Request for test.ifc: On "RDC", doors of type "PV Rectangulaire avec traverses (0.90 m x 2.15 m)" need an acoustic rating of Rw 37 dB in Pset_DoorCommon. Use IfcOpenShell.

First a look at what the model holds.

```python
import ifcopenshell
import ifcopenshell.util.element

model = ifcopenshell.open("test.ifc")
print(model.schema)
storey = next(s for s in model.by_type("IfcBuildingStorey") if s.Name == "RDC")
doors = [e for e in ifcopenshell.util.element.get_decomposition(storey) if e.is_a("IfcDoor")]
seen = {}
for e in doors:
    element_type = ifcopenshell.util.element.get_type(e)
    key = (element_type.Name if element_type != e and element_type else None, ifcopenshell.util.element.get_pset(e, "Pset_DoorCommon", "AcousticRating"))
    seen[key] = seen.get(key, 0) + 1
for (name, value), count in sorted(seen.items(), key=str):
    print(count, "x", name, "|", value)
```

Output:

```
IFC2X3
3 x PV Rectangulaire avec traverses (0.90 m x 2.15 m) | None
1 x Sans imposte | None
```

```python
import ifcopenshell
import ifcopenshell.api.pset
import ifcopenshell.util.element

model = ifcopenshell.open("test.ifc")

storey = next(s for s in model.by_type("IfcBuildingStorey") if s.Name == "RDC")
doors = [e for e in ifcopenshell.util.element.get_decomposition(storey) if e.is_a("IfcDoor")]

count = 0
for e in doors:
    element_type = ifcopenshell.util.element.get_type(e)
    if element_type in (None, e) or element_type.Name != "PV Rectangulaire avec traverses (0.90 m x 2.15 m)":
        continue
    # add_pset returns the element's existing set when there is one.
    pset = ifcopenshell.api.pset.add_pset(model, product=e, name="Pset_DoorCommon")
    ifcopenshell.api.pset.edit_pset(model, pset=pset, properties={"AcousticRating": "Rw 37 dB"})
    count += 1

print(count, "doors updated")

model.write("test_rev.ifc")
```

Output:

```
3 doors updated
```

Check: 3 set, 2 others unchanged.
